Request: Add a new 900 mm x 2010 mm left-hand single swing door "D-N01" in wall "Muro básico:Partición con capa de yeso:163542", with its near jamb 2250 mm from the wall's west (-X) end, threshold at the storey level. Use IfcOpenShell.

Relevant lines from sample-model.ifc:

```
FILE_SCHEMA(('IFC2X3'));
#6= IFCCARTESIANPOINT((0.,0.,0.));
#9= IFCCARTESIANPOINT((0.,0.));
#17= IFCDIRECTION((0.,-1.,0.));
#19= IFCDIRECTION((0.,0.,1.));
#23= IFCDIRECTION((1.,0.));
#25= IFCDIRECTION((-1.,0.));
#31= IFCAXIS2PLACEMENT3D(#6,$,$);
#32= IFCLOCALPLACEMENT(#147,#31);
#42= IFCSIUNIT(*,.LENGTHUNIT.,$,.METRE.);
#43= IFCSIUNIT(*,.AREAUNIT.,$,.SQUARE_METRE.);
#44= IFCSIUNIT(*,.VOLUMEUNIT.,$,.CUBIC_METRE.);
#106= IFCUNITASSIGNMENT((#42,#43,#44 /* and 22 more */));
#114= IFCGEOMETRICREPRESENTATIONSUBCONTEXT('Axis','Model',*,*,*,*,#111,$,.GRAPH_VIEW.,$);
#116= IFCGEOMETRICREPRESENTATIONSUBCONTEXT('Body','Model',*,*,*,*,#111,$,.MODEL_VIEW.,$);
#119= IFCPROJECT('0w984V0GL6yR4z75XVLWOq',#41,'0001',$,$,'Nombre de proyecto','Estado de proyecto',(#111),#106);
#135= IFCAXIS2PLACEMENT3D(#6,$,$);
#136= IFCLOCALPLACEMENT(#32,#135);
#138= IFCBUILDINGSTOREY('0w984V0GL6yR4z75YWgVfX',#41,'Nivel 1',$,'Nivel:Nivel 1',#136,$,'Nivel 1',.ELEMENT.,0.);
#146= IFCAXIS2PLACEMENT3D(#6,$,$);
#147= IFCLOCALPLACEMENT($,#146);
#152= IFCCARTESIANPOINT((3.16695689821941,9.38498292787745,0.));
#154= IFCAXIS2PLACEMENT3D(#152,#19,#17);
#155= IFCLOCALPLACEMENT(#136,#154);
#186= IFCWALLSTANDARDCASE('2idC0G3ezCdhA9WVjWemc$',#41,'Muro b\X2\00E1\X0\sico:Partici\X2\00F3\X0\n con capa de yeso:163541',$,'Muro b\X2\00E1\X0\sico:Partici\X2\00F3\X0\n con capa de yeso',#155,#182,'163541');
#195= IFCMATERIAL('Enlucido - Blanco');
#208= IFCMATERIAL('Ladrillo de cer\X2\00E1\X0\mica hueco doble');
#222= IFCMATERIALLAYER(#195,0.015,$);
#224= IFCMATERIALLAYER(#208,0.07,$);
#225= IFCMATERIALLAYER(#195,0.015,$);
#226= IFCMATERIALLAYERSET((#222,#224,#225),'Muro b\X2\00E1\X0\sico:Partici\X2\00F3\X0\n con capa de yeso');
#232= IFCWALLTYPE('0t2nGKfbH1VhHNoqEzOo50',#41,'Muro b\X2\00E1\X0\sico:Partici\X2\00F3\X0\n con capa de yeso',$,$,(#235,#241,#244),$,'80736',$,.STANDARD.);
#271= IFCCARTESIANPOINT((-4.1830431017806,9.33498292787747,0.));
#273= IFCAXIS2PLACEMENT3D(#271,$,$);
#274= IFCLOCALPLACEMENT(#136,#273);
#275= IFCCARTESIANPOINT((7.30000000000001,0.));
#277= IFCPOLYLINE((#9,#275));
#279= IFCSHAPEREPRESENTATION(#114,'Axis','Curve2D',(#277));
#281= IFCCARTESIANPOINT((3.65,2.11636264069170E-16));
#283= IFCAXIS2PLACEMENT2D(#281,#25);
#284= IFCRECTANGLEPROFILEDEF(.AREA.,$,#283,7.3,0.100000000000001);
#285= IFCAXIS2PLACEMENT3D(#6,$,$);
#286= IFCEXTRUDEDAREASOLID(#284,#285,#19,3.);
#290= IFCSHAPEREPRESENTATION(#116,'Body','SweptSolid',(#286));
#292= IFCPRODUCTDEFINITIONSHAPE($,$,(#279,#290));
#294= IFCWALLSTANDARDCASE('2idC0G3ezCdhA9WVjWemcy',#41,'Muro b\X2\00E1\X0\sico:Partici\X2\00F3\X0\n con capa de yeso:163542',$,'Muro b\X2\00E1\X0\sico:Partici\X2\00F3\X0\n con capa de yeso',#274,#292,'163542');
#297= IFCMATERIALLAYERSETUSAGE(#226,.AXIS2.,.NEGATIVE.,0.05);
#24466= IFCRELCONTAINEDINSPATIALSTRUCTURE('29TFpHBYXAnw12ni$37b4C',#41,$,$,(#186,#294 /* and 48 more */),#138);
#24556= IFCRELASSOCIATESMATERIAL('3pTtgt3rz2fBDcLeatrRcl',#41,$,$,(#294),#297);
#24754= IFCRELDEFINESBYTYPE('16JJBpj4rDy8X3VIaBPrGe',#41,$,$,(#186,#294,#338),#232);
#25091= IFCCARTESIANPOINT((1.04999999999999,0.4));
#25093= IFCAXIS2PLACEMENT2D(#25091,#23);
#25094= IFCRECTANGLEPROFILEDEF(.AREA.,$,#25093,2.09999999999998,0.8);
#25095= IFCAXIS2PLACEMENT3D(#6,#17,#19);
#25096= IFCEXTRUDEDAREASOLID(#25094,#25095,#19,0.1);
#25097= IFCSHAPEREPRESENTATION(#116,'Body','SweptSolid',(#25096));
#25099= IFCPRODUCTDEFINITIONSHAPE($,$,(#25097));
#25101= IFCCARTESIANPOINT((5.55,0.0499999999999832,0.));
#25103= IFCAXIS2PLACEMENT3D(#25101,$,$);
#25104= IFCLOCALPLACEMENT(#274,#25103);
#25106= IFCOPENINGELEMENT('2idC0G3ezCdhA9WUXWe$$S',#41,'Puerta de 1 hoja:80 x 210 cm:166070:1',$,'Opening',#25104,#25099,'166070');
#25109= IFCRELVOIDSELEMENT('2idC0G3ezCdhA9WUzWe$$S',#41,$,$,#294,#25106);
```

```python
import numpy as np
import ifcopenshell
import ifcopenshell.api.feature
import ifcopenshell.api.geometry
import ifcopenshell.api.root
import ifcopenshell.api.spatial
import ifcopenshell.api.type
import ifcopenshell.geom
import ifcopenshell.util.element
import ifcopenshell.util.placement
import ifcopenshell.util.representation
import ifcopenshell.util.shape
import ifcopenshell.util.unit

model = ifcopenshell.open("sample-model.ifc")
unit_scale = ifcopenshell.util.unit.calculate_unit_scale(model)
settings = ifcopenshell.geom.settings()


def volume(element):
    """Net volume in cubic metres, openings subtracted."""
    shape = ifcopenshell.geom.create_shape(settings, element)
    return ifcopenshell.util.shape.get_volume(shape.geometry)


wall = model.by_id(294)
storey = ifcopenshell.util.element.get_container(wall, ifc_class="IfcBuildingStorey")
context = ifcopenshell.util.representation.get_context(model, "Model", "Body", "MODEL_VIEW")
before = volume(wall)

width, height, from_end, sill = 0.9, 2.01, 2.25, 0.0  # metres

# The wall runs along its own X axis, and the end named is its -X end.
wall_shape = ifcopenshell.geom.create_shape(settings, wall)
x, y, z = ifcopenshell.util.shape.get_vertices(wall_shape.geometry).T
start = x.min() + from_end
face, thickness = float(y.min()), float(y.max() - y.min())
wall_matrix = ifcopenshell.util.placement.get_local_placement(wall.ObjectPlacement)
level = ifcopenshell.util.placement.get_local_placement(storey.ObjectPlacement)[2, 3]


def in_wall(x, y):
    """Placement at x, y metres in the wall's axes, at sill height."""
    matrix = wall_matrix.copy()
    matrix[:, 3] = wall_matrix @ np.array([x / unit_scale, y / unit_scale, 0.0, 1.0])
    matrix[2, 3] = level + sill / unit_scale
    return matrix


# Opening: a box that overshoots both wall faces by 50 mm.
opening = ifcopenshell.api.root.create_entity(model, ifc_class="IfcOpeningElement")
box = ifcopenshell.api.geometry.add_wall_representation(
    model, context=context, length=width, height=height, thickness=thickness + 0.1
)
ifcopenshell.api.geometry.assign_representation(model, product=opening, representation=box)
ifcopenshell.api.geometry.edit_object_placement(model, product=opening, matrix=in_wall(start, face - 0.05), is_si=False)
ifcopenshell.api.feature.add_feature(model, feature=opening, element=wall)

door = ifcopenshell.api.root.create_entity(model, ifc_class="IfcDoor", name="D-N01")
door.OverallWidth, door.OverallHeight = width / unit_scale, height / unit_scale
body = ifcopenshell.api.geometry.add_door_representation(
    model,
    context=context,
    overall_width=door.OverallWidth,
    overall_height=door.OverallHeight,
    operation_type="SINGLE_SWING_LEFT",
    lining_properties={"LiningDepth": thickness / unit_scale, "ThresholdDepth": thickness / unit_scale},
)
ifcopenshell.api.geometry.assign_representation(model, product=door, representation=body)
ifcopenshell.api.spatial.assign_container(model, products=[door], relating_structure=storey)
fills = ifcopenshell.api.feature.add_filling(model, opening=opening, element=door)
fills.OwnerHistory = door.OwnerHistory  # required in IFC2X3

# IFC2X3 keeps the operation on the door style.
style = ifcopenshell.api.root.create_entity(model, ifc_class="IfcDoorStyle", name="D-N01")
style.OperationType, style.ConstructionType = "SINGLE_SWING_LEFT", "NOTDEFINED"
style.ParameterTakesPrecedence = style.Sizeable = False
ifcopenshell.api.type.assign_type(model, related_objects=[door], relating_type=style)

# The lining spans the wall, so the door starts at the wall face.
ifcopenshell.api.geometry.edit_object_placement(model, product=door, matrix=in_wall(start, face), is_si=False)

after = volume(wall)

print(f"wall volume {before:.3f} -> {after:.3f} m3")

model.write("sample-model_rev.ifc")
```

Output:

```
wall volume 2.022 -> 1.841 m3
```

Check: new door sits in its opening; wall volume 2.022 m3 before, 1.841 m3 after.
